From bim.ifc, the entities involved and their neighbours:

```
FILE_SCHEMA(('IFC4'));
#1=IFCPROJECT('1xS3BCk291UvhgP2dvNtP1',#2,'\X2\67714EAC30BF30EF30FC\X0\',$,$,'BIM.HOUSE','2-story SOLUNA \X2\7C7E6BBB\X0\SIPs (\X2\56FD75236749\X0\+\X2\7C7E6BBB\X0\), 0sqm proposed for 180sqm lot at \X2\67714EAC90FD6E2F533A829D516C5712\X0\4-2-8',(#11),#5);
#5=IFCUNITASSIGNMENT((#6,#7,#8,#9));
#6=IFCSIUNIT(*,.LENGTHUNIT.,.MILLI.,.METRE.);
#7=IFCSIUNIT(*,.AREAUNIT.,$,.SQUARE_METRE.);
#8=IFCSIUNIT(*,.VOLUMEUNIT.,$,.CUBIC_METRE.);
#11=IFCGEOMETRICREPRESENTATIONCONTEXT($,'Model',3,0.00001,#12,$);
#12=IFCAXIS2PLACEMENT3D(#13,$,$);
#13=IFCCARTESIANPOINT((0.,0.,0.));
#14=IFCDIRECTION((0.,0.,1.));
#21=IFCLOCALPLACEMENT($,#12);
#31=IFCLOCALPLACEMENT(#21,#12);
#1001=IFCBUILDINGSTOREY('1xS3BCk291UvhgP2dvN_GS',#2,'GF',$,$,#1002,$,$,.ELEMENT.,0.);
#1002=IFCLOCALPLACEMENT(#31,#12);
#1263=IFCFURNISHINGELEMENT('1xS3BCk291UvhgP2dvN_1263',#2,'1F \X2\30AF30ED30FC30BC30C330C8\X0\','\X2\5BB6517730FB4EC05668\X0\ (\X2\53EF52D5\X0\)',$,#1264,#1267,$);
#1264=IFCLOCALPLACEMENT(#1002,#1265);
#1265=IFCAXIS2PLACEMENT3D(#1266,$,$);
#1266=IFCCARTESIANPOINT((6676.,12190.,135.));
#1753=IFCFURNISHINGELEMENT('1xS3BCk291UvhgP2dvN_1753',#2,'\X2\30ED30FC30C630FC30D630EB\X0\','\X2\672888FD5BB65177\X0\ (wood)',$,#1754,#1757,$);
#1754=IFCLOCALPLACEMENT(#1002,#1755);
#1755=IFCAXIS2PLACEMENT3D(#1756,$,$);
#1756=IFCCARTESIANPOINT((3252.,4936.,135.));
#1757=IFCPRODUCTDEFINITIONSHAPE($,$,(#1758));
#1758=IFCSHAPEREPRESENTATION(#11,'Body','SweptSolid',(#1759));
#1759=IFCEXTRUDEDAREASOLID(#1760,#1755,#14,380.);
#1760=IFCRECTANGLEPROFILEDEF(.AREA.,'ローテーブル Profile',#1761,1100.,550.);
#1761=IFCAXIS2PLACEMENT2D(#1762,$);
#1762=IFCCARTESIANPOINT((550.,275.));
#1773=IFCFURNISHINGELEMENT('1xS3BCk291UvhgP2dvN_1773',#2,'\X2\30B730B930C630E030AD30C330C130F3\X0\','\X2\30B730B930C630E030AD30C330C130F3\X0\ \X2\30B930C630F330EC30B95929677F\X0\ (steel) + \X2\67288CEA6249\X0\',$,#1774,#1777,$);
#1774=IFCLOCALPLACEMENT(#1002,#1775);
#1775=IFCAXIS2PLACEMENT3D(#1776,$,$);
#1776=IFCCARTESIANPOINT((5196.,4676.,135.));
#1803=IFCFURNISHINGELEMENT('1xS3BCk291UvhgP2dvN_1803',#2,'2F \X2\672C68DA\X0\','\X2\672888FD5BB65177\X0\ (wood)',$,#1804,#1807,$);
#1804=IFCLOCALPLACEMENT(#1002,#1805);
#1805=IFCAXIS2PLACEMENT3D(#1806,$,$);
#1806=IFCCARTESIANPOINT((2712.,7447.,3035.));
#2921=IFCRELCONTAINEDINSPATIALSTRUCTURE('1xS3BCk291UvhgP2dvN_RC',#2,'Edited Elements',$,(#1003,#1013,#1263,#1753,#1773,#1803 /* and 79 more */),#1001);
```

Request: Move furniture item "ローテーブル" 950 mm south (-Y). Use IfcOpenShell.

```python
import ifcopenshell
import ifcopenshell.api.geometry
import ifcopenshell.util.placement

model = ifcopenshell.open("bim.ifc")

item = model.by_guid("1xS3BCk291UvhgP2dvN_1753")
matrix = ifcopenshell.util.placement.get_local_placement(item.ObjectPlacement)
matrix[1, 3] -= 950.0
ifcopenshell.api.geometry.edit_object_placement(model, product=item, matrix=matrix, is_si=False)

print(ifcopenshell.util.placement.get_local_placement(item.ObjectPlacement).round(3) + 0.0)

model.write("bim_edited.ifc")
```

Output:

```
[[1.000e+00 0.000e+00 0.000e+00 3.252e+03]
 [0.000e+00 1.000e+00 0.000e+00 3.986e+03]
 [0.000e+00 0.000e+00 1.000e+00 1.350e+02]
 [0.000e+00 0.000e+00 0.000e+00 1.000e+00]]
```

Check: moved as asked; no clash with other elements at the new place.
